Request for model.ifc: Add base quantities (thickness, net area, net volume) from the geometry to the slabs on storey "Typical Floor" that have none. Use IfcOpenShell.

First a look at what the model holds.

```python
import ifcopenshell
import ifcopenshell.util.element
import ifcopenshell.util.unit

model = ifcopenshell.open("model.ifc")
print(model.schema)
for unit_type in ("LENGTHUNIT", "AREAUNIT", "VOLUMEUNIT"):
    print(unit_type, ifcopenshell.util.unit.calculate_unit_scale(model, unit_type))
storey = next(s for s in model.by_type("IfcBuildingStorey") if s.Name == "Typical Floor")
slabs = [e for e in ifcopenshell.util.element.get_decomposition(storey) if e.is_a("IfcSlab")]
for e in sorted(slabs, key=lambda e: e.id()):
    print(e.id(), e.is_a(), e.Name, list(ifcopenshell.util.element.get_psets(e, qtos_only=True)), sep=" | ")
```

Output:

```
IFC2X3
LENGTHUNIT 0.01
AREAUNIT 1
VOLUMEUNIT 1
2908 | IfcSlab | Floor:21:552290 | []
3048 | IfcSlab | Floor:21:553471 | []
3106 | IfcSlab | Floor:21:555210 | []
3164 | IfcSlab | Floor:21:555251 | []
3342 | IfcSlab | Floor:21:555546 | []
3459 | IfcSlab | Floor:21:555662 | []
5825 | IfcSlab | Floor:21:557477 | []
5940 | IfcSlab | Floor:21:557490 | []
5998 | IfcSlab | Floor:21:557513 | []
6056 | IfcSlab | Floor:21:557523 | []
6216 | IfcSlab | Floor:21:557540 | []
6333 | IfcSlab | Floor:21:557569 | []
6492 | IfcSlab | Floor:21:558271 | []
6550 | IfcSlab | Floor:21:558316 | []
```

```python
import ifcopenshell
import ifcopenshell.api.pset
import ifcopenshell.geom
import ifcopenshell.util.element
import ifcopenshell.util.shape
import ifcopenshell.util.unit

model = ifcopenshell.open("model.ifc")
unit_scale = ifcopenshell.util.unit.calculate_unit_scale(model)
area_scale = ifcopenshell.util.unit.calculate_unit_scale(model, "AREAUNIT")
volume_scale = ifcopenshell.util.unit.calculate_unit_scale(model, "VOLUMEUNIT")
settings = ifcopenshell.geom.settings()

storey = next(s for s in model.by_type("IfcBuildingStorey") if s.Name == "Typical Floor")
slabs = [e for e in ifcopenshell.util.element.get_decomposition(storey) if e.is_a("IfcSlab")]

for e in sorted(slabs, key=lambda e: e.id()):
    if ifcopenshell.util.element.get_psets(e, qtos_only=True, should_inherit=False):
        continue
    # Geometry comes back in metres, in the element's own axes.
    shape = ifcopenshell.geom.create_shape(settings, e)
    values = {
        "Width": ifcopenshell.util.shape.get_z(shape.geometry) / unit_scale,
        "NetArea": ifcopenshell.util.shape.get_footprint_area(shape.geometry) / area_scale,
        "NetVolume": ifcopenshell.util.shape.get_volume(shape.geometry) / volume_scale,
    }
    qto = ifcopenshell.api.pset.add_qto(model, product=e, name="BaseQuantities")
    ifcopenshell.api.pset.edit_qto(model, qto=qto, properties=values)
    print(e.id(), {k: round(v, 3) for k, v in values.items()})

model.write("model_edited.ifc")
```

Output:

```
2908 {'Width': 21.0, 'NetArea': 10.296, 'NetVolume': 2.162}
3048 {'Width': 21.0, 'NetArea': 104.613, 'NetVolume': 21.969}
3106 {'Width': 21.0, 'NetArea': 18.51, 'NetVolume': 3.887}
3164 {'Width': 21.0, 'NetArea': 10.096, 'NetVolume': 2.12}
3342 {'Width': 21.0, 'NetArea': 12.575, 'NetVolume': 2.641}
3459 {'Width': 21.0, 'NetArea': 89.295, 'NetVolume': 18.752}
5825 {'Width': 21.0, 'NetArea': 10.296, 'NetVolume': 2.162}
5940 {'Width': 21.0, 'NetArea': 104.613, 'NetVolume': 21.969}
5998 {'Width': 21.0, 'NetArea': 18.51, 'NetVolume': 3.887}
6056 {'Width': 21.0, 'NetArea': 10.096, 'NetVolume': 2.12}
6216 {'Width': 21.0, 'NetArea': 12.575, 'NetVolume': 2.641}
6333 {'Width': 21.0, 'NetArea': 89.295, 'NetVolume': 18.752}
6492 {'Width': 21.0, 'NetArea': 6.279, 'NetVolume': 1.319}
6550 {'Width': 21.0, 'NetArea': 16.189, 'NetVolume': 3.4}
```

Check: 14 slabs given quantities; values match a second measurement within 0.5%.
